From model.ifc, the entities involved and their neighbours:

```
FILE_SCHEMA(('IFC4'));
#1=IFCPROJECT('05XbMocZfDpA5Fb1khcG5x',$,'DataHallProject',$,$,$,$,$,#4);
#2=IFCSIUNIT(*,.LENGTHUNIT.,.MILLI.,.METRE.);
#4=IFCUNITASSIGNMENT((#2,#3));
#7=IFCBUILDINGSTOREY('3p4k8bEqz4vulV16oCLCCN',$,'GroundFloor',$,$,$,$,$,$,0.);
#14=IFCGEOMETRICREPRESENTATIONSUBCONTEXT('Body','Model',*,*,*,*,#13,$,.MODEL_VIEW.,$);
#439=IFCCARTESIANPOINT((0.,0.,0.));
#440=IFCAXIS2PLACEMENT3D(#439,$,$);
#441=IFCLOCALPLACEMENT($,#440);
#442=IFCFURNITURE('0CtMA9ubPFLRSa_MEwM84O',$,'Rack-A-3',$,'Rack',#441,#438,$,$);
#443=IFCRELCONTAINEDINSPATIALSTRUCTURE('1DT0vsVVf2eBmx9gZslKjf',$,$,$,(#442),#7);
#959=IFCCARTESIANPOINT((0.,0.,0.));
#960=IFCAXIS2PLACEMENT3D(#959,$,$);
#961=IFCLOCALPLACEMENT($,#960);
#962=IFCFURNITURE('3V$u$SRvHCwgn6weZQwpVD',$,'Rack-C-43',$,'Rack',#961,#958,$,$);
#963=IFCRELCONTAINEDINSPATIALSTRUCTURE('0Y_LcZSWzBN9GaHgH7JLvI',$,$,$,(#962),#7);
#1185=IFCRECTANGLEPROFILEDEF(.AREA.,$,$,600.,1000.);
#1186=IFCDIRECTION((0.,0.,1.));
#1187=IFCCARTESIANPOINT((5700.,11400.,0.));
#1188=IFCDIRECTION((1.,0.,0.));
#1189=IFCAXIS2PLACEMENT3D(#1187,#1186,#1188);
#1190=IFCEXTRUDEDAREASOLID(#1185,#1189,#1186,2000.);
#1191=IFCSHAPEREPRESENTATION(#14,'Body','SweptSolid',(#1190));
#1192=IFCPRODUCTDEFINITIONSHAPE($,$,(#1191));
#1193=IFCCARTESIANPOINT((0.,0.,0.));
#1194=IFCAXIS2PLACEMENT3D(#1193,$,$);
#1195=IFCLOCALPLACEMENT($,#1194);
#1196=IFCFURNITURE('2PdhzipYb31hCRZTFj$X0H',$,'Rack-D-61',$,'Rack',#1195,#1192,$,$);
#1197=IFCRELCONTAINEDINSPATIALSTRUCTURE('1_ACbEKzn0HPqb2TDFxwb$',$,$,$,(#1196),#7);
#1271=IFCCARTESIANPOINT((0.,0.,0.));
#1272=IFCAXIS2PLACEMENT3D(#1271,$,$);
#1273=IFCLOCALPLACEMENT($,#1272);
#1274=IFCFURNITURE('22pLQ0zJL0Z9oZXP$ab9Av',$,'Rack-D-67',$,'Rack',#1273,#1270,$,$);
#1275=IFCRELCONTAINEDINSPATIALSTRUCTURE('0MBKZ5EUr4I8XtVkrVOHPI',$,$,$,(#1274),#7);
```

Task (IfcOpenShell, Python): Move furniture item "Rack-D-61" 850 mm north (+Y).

```python
import ifcopenshell
import ifcopenshell.api.geometry
import ifcopenshell.util.placement
import ifcopenshell.util.unit

model = ifcopenshell.open("model.ifc")
unit_scale = ifcopenshell.util.unit.calculate_unit_scale(model)

item = model.by_guid("2PdhzipYb31hCRZTFj$X0H")
matrix = ifcopenshell.util.placement.get_local_placement(item.ObjectPlacement)
matrix[1, 3] += 0.85 / unit_scale
ifcopenshell.api.geometry.edit_object_placement(model, product=item, matrix=matrix, is_si=False)

print(ifcopenshell.util.placement.get_local_placement(item.ObjectPlacement).round(3) + 0.0)

model.write("model_v2.ifc")
```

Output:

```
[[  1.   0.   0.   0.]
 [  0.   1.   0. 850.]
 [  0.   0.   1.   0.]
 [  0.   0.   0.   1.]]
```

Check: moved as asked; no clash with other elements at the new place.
